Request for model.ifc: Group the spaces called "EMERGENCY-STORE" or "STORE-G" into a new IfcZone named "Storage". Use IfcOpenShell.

First a look at what the model holds.

```python
import ifcopenshell

model = ifcopenshell.open("model.ifc")
print(model.schema)
seen = {}
for space in model.by_type("IfcSpace"):
    seen[space.Name] = seen.get(space.Name, 0) + 1
for name, count in sorted(seen.items(), key=str):
    print(count, "x", name)
print("zones:", [z.Name for z in model.by_type("IfcZone")][:20])
```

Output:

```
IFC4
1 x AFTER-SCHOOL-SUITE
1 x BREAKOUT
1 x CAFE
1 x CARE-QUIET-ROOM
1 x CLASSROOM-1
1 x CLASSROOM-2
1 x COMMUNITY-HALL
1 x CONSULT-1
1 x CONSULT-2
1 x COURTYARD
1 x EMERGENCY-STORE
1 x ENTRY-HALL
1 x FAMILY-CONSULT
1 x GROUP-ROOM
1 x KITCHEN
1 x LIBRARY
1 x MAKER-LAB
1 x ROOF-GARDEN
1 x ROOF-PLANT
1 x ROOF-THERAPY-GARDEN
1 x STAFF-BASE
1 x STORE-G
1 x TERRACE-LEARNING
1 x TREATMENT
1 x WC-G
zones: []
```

```python
import ifcopenshell
import ifcopenshell.api.group
import ifcopenshell.api.root

model = ifcopenshell.open("model.ifc")

names = {"EMERGENCY-STORE", "STORE-G"}
spaces = [s for s in model.by_type("IfcSpace") if s.Name in names]

zone = ifcopenshell.api.root.create_entity(model, ifc_class="IfcZone", name="Storage")
ifcopenshell.api.group.assign_group(model, products=spaces, group=zone)
print(len(spaces), "spaces in", zone.Name)

model.write("model-out.ifc")
```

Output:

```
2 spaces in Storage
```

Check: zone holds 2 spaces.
